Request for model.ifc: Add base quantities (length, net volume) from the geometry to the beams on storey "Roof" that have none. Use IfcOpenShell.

First a look at what the model holds.

```python
import ifcopenshell
import ifcopenshell.util.element
import ifcopenshell.util.unit

model = ifcopenshell.open("model.ifc")
print(model.schema)
for unit_type in ("LENGTHUNIT", "AREAUNIT", "VOLUMEUNIT"):
    print(unit_type, ifcopenshell.util.unit.calculate_unit_scale(model, unit_type))
storey = next(s for s in model.by_type("IfcBuildingStorey") if s.Name == "Roof")
beams = [e for e in ifcopenshell.util.element.get_decomposition(storey) if e.is_a("IfcBeam")]
for e in sorted(beams, key=lambda e: e.id()):
    print(e.id(), e.is_a(), e.Name, list(ifcopenshell.util.element.get_psets(e, qtos_only=True)), sep=" | ")
```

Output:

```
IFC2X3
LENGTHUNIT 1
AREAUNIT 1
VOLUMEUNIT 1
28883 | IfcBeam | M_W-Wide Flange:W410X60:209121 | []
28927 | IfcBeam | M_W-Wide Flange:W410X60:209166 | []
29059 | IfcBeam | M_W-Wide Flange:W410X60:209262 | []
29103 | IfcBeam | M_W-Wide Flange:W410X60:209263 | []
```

```python
import ifcopenshell
import ifcopenshell.api.pset
import ifcopenshell.geom
import ifcopenshell.util.element
import ifcopenshell.util.shape
import ifcopenshell.util.unit

model = ifcopenshell.open("model.ifc")
unit_scale = ifcopenshell.util.unit.calculate_unit_scale(model)
volume_scale = ifcopenshell.util.unit.calculate_unit_scale(model, "VOLUMEUNIT")
settings = ifcopenshell.geom.settings()

storey = next(s for s in model.by_type("IfcBuildingStorey") if s.Name == "Roof")
beams = [e for e in ifcopenshell.util.element.get_decomposition(storey) if e.is_a("IfcBeam")]

for e in sorted(beams, key=lambda e: e.id()):
    if ifcopenshell.util.element.get_psets(e, qtos_only=True, should_inherit=False):
        continue
    # Geometry comes back in metres, in the element's own axes.
    shape = ifcopenshell.geom.create_shape(settings, e)
    values = {
        "Length": ifcopenshell.util.shape.get_max_xyz(shape.geometry) / unit_scale,
        "NetVolume": ifcopenshell.util.shape.get_volume(shape.geometry) / volume_scale,
    }
    qto = ifcopenshell.api.pset.add_qto(model, product=e, name="BaseQuantities")
    ifcopenshell.api.pset.edit_qto(model, qto=qto, properties=values)
    print(e.id(), {k: round(v, 3) for k, v in values.items()})

model.write("model_v2.ifc")
```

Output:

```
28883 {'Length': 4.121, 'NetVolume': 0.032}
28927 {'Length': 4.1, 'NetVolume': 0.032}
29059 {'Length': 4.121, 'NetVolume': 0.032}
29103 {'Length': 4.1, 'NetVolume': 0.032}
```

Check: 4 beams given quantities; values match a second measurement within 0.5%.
